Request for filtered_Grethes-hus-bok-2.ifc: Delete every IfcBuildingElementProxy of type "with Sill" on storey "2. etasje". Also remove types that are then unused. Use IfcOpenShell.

First a look at what the model holds.

```python
import ifcopenshell
import ifcopenshell.util.element

model = ifcopenshell.open("filtered_Grethes-hus-bok-2.ifc")
print(model.schema)
storey = next(s for s in model.by_type("IfcBuildingStorey") if s.Name == "2. etasje")
proxies = [e for e in ifcopenshell.util.element.get_decomposition(storey) if e.is_a("IfcBuildingElementProxy")]
seen = {}
for e in proxies:
    element_type = ifcopenshell.util.element.get_type(e)
    name = element_type.Name if element_type not in (None, e) else None
    seen[name] = seen.get(name, 0) + 1
for name, count in sorted(seen.items(), key=str):
    print(count, "x", name)
```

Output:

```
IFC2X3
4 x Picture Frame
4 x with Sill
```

```python
import ifcopenshell
import ifcopenshell.api.root
import ifcopenshell.util.element

model = ifcopenshell.open("filtered_Grethes-hus-bok-2.ifc")

storey = next(s for s in model.by_type("IfcBuildingStorey") if s.Name == "2. etasje")
proxies = [e for e in ifcopenshell.util.element.get_decomposition(storey) if e.is_a("IfcBuildingElementProxy")]
targets = [e for e in proxies if (t := ifcopenshell.util.element.get_type(e)) not in (None, e) and t.Name == "with Sill"]
types = {ifcopenshell.util.element.get_type(e) for e in targets} - {None, *targets}

for e in targets:
    ifcopenshell.api.root.remove_product(model, product=e)
print(len(targets), "removed")

unused = [t for t in types if not ifcopenshell.util.element.get_types(t)]
for t in unused:
    ifcopenshell.api.root.remove_product(model, product=t)
print(len(unused), "unused types removed")

model.write("filtered_Grethes-hus-bok-2_v2.ifc")
```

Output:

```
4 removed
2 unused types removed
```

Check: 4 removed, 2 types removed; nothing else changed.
